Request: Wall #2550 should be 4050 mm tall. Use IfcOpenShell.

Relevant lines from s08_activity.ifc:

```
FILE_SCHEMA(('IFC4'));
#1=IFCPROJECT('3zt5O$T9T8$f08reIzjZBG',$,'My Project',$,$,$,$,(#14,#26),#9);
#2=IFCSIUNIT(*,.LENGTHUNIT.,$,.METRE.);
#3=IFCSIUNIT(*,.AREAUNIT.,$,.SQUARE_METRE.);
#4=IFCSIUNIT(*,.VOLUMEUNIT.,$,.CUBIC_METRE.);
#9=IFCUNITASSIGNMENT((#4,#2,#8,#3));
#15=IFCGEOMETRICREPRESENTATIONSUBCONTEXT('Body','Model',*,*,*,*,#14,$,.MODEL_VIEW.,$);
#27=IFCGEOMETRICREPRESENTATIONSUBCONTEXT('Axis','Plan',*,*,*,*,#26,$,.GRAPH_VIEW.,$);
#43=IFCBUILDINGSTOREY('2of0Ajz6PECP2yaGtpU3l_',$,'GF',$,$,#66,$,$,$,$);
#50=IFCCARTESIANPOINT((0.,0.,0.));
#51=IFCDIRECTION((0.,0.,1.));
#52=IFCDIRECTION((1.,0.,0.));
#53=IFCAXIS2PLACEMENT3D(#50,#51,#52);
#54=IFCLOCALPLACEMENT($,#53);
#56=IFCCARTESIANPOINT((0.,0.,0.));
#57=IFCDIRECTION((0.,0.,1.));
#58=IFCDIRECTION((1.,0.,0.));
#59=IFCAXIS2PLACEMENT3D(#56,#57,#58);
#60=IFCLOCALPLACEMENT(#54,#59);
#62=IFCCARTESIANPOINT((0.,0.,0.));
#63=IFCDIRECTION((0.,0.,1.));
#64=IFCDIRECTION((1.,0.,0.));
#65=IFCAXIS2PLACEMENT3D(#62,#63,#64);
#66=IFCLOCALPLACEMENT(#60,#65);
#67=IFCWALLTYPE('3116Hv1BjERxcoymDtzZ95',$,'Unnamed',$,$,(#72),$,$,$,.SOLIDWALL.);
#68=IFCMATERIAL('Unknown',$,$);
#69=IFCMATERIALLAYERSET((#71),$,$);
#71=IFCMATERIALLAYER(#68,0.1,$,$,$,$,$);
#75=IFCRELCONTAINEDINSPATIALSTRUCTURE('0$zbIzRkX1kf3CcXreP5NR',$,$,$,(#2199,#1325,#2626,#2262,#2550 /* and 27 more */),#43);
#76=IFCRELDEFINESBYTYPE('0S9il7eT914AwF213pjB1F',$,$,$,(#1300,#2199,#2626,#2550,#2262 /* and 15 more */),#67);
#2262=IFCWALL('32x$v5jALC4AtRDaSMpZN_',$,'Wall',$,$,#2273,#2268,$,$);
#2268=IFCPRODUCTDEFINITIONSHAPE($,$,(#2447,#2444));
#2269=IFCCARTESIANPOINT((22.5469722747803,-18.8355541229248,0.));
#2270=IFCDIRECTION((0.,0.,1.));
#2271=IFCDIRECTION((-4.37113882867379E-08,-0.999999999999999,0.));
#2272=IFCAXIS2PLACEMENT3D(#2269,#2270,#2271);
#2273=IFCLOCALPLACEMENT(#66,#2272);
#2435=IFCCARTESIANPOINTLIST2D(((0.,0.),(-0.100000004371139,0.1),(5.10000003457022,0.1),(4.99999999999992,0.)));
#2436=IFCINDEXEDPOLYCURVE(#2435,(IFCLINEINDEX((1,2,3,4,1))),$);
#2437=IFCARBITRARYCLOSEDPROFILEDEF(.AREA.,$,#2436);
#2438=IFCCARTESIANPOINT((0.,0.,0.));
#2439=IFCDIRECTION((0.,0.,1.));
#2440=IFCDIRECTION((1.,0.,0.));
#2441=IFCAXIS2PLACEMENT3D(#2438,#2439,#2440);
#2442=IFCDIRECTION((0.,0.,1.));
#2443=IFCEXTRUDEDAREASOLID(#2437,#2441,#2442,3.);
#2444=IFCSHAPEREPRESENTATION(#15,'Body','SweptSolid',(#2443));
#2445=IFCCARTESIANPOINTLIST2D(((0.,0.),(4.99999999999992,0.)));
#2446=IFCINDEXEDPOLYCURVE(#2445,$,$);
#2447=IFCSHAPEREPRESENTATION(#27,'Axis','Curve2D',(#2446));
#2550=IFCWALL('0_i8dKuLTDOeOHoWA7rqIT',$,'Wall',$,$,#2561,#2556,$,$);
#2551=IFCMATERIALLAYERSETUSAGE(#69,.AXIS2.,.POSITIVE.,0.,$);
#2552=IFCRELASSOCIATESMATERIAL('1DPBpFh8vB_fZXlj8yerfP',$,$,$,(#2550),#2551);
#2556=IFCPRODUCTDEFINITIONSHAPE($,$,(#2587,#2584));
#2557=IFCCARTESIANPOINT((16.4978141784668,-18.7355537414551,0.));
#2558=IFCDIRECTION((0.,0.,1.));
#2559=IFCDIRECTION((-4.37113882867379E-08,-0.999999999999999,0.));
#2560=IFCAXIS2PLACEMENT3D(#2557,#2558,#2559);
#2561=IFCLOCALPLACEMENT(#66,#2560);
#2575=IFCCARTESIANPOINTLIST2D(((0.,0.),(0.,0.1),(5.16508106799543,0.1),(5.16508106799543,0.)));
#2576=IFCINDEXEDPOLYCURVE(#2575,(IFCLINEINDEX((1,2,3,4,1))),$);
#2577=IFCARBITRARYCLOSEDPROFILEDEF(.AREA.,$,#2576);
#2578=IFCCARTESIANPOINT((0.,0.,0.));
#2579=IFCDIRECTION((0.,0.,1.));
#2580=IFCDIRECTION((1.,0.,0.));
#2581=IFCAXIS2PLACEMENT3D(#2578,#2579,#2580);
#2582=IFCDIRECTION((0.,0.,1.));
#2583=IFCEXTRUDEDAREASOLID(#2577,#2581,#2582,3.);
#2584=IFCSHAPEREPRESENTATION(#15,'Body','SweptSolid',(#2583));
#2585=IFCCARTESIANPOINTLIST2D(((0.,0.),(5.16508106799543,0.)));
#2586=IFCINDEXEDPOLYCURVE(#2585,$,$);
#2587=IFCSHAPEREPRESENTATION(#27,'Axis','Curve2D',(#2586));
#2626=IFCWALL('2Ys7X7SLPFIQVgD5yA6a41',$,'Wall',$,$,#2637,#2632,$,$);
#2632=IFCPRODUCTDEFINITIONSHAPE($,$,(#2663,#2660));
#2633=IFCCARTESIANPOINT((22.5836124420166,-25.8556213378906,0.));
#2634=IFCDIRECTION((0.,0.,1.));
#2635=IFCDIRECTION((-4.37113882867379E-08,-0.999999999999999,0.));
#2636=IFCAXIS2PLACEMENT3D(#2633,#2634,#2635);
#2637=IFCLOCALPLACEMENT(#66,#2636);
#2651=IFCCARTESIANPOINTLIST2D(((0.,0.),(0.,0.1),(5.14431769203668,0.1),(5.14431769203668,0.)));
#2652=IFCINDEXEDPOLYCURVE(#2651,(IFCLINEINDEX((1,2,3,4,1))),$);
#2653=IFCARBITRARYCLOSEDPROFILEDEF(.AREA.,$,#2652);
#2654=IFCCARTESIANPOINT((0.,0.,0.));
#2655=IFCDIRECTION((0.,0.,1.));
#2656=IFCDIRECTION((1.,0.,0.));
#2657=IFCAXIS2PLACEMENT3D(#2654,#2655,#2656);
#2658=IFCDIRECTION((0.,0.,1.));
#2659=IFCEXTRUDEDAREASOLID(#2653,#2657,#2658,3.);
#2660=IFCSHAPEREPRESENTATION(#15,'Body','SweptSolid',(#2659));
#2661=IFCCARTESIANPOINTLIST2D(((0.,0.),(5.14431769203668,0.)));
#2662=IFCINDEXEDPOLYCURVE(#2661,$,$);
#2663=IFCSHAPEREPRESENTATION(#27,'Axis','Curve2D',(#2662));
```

```python
import ifcopenshell
import ifcopenshell.geom
import ifcopenshell.util.representation
import ifcopenshell.util.shape
import ifcopenshell.util.unit

model = ifcopenshell.open("s08_activity.ifc")
unit_scale = ifcopenshell.util.unit.calculate_unit_scale(model)
settings = ifcopenshell.geom.settings()


def volume(element):
    """Net volume in cubic metres, openings subtracted."""
    shape = ifcopenshell.geom.create_shape(settings, element)
    return ifcopenshell.util.shape.get_volume(shape.geometry)


wall = model.by_guid("0_i8dKuLTDOeOHoWA7rqIT")
before = volume(wall)

body = ifcopenshell.util.representation.get_representation(wall, "Model", "Body")
solid = body.Items[0]
old_height = solid.Depth
solid.Depth = 4.05 / unit_scale
after = volume(wall)

print(f"height {old_height:g} -> {solid.Depth:g}, volume {before:.3f} -> {after:.3f} m3")

model.write("s08_activity_updated.ifc")
```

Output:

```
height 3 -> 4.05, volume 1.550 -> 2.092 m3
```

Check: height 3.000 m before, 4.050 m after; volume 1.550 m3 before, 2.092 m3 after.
